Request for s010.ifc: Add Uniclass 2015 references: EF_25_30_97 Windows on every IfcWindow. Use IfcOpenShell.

First a look at what the model holds.

```python
import ifcopenshell

model = ifcopenshell.open("s010.ifc")
print(model.schema)
print("classifications:", [c.Name for c in model.by_type("IfcClassification")])
for ifc_class in ("IfcDoor", "IfcRoof", "IfcStair", "IfcWall", "IfcWindow"):
    print(ifc_class, len(model.by_type(ifc_class)))
```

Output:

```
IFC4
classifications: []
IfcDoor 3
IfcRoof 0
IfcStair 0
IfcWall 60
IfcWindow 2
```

```python
import ifcopenshell
import ifcopenshell.api.classification

model = ifcopenshell.open("s010.ifc")

system = ifcopenshell.api.classification.add_classification(model, classification="Uniclass 2015")

codes = {
    "IfcWindow": ("EF_25_30_97", "Windows"),
}
for ifc_class, (code, name) in codes.items():
    products = model.by_type(ifc_class)
    ifcopenshell.api.classification.add_reference(
        model, products=products, classification=system, identification=code, name=name
    )
    print(code, len(products))

model.write("s010_edited.ifc")
```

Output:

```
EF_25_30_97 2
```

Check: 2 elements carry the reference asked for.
